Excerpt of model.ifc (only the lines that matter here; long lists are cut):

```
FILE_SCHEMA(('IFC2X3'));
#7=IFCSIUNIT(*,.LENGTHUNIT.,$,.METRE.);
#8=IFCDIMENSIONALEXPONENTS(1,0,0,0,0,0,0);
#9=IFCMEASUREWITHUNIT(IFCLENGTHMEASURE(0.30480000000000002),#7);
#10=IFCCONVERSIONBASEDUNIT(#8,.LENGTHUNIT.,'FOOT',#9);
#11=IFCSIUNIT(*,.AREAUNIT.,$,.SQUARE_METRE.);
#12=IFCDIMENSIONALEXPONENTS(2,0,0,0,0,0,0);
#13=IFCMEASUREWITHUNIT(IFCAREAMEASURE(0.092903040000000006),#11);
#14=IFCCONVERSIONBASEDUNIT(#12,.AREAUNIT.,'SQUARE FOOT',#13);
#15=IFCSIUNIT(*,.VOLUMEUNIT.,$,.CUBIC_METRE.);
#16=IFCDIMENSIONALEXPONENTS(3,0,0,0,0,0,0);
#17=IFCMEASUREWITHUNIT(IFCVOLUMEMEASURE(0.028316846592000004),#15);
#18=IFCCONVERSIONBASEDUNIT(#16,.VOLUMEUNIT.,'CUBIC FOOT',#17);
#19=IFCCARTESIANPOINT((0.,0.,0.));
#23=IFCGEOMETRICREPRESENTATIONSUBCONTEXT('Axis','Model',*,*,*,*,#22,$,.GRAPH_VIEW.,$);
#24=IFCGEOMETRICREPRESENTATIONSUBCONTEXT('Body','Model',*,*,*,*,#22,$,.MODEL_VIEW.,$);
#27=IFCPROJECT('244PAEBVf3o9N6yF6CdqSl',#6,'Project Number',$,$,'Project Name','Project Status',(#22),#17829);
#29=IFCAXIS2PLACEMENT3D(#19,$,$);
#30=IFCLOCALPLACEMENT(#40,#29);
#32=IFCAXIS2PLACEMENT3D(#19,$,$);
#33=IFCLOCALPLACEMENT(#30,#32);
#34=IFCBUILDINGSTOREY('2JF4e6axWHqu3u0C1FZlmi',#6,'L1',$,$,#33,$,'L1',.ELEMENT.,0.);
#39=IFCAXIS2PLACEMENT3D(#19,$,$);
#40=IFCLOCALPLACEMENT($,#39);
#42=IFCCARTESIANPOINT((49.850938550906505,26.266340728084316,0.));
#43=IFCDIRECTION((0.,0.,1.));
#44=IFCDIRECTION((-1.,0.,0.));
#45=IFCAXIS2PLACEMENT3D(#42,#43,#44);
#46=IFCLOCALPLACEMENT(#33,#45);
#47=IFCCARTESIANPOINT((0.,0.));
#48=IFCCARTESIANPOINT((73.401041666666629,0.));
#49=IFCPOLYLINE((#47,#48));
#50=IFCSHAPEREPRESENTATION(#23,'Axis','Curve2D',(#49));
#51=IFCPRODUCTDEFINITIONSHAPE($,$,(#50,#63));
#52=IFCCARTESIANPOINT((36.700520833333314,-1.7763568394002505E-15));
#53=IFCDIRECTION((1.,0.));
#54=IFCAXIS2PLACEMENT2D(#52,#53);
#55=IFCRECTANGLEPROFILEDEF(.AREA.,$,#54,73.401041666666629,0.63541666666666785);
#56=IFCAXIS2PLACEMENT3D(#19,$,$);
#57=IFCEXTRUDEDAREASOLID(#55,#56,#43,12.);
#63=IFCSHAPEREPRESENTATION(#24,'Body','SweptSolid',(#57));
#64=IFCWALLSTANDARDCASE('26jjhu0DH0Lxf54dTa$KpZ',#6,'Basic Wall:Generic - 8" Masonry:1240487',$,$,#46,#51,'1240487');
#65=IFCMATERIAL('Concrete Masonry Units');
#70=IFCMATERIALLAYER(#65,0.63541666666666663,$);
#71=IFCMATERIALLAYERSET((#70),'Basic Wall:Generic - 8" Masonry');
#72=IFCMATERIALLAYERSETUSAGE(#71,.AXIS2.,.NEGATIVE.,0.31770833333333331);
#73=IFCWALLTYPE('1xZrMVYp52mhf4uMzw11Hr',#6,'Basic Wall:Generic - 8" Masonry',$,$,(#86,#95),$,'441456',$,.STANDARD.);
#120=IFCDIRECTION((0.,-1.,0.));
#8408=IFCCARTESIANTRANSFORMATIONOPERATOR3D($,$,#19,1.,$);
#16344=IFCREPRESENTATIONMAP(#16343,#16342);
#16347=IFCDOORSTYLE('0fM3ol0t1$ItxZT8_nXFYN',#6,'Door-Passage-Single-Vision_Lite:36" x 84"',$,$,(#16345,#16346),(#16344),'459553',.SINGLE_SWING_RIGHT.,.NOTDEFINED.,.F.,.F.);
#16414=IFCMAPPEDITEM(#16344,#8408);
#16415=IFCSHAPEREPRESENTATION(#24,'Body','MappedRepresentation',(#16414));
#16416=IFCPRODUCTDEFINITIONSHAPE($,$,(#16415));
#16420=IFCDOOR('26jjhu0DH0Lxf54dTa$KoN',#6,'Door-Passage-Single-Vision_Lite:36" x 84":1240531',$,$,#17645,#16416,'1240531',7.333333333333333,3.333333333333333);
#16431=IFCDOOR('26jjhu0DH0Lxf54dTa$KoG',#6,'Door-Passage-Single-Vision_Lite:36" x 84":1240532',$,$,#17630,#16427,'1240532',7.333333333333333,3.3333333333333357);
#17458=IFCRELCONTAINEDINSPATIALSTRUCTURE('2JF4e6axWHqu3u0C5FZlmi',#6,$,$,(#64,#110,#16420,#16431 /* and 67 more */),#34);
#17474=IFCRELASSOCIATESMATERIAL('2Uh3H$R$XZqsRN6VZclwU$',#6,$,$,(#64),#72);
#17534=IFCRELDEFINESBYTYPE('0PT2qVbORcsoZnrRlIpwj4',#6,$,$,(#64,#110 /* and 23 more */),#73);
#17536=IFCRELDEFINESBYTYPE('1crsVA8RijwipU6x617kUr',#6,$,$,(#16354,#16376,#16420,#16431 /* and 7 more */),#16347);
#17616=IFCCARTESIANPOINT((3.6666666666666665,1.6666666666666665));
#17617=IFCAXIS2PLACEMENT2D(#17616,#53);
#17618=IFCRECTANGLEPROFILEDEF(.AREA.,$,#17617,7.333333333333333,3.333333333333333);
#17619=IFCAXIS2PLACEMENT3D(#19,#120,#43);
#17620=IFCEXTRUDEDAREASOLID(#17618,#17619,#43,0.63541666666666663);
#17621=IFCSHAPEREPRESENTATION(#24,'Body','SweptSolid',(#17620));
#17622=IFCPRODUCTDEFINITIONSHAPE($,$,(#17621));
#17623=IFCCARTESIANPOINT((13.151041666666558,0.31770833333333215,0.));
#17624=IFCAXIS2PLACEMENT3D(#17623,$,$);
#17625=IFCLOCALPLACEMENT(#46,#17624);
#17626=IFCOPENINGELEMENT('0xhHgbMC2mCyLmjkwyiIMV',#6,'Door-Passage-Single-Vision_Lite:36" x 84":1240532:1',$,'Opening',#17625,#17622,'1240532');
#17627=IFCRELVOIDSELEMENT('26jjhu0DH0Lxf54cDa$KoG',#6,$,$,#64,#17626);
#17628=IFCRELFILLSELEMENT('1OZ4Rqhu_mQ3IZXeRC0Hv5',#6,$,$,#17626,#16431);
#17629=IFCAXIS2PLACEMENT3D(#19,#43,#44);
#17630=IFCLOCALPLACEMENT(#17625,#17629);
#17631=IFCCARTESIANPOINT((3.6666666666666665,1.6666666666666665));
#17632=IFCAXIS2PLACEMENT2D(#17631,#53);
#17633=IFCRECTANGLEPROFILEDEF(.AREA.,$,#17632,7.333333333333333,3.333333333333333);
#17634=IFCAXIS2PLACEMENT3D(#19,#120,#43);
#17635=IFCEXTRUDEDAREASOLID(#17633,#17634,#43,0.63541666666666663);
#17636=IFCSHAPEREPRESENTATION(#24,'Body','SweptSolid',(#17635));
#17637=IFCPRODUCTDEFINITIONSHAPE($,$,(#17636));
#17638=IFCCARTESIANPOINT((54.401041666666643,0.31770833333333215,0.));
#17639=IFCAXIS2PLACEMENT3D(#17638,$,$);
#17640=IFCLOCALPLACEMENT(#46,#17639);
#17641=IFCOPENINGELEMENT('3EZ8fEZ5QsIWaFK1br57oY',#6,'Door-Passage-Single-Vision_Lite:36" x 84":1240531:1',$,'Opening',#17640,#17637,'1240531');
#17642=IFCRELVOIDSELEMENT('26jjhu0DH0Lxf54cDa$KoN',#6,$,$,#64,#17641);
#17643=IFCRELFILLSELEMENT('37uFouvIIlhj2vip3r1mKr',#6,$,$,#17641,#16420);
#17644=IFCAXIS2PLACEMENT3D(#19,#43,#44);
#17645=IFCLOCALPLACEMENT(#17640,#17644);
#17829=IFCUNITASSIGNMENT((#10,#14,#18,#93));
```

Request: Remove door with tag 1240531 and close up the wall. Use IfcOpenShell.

```python
import ifcopenshell
import ifcopenshell.api.feature
import ifcopenshell.api.root
import ifcopenshell.geom
import ifcopenshell.util.shape

model = ifcopenshell.open("model.ifc")
settings = ifcopenshell.geom.settings()


def volume(element):
    """Net volume in cubic metres, openings subtracted."""
    shape = ifcopenshell.geom.create_shape(settings, element)
    return ifcopenshell.util.shape.get_volume(shape.geometry)


door = model.by_guid("26jjhu0DH0Lxf54dTa$KoN")
opening = door.FillsVoids[0].RelatingOpeningElement
wall = opening.VoidsElements[0].RelatingBuildingElement
before = volume(wall)

ifcopenshell.api.root.remove_product(model, product=door)
ifcopenshell.api.feature.remove_feature(model, feature=opening)

after = volume(wall)

print(f"wall volume {before:.3f} -> {after:.3f} m3")

model.write("model-out.ifc")
```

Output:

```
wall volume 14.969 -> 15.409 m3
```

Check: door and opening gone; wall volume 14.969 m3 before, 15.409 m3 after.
